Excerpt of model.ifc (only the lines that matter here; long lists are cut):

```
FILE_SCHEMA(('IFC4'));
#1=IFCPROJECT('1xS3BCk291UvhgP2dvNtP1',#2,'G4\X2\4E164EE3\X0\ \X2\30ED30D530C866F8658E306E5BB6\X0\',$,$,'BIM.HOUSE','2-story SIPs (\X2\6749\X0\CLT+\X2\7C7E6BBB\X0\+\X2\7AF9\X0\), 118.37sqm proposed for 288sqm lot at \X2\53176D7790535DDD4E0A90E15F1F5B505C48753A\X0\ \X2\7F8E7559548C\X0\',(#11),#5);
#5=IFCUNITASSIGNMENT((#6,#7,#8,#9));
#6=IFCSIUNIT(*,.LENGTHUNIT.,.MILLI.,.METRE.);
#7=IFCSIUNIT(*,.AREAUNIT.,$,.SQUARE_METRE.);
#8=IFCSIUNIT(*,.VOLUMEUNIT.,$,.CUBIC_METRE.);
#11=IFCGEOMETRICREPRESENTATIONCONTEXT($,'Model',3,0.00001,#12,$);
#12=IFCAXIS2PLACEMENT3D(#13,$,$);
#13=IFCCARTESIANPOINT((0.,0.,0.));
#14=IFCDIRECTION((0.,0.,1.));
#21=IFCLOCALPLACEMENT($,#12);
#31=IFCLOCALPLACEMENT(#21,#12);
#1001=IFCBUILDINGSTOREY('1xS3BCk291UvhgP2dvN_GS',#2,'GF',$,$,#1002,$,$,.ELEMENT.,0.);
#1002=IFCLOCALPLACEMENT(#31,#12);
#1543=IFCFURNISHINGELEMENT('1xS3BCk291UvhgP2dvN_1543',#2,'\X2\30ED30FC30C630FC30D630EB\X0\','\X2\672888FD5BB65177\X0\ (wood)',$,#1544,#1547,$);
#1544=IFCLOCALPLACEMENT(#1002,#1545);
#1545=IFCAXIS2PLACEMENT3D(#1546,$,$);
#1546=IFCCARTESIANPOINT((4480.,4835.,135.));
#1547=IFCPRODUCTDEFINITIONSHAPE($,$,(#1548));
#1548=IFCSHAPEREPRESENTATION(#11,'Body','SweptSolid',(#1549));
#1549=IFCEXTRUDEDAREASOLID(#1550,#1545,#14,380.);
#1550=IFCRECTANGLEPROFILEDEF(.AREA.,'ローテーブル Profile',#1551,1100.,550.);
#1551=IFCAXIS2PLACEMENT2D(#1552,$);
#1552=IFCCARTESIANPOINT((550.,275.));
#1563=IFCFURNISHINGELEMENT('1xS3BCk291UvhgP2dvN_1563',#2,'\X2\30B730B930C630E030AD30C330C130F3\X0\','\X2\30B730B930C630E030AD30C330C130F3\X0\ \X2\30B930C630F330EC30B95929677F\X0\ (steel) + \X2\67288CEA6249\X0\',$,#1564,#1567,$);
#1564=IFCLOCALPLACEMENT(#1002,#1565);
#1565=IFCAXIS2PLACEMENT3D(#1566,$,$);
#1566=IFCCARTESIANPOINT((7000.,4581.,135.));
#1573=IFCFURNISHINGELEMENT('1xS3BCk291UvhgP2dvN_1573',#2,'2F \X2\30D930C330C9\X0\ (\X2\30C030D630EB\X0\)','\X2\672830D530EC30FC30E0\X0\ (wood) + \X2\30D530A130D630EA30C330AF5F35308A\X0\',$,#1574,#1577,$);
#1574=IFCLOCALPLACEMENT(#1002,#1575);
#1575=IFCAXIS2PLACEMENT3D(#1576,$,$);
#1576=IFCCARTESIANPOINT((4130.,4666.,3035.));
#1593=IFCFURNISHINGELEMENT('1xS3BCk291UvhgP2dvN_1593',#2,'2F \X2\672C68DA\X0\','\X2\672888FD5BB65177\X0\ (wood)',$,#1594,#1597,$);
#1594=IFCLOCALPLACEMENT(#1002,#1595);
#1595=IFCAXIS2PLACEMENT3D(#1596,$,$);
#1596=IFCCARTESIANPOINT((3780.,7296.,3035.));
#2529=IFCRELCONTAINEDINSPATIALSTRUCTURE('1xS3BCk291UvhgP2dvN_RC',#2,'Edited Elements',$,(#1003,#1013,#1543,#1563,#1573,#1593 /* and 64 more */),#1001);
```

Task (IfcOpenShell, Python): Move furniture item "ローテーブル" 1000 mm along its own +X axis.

```python
import ifcopenshell
import ifcopenshell.api.geometry
import ifcopenshell.util.placement
import ifcopenshell.util.unit

model = ifcopenshell.open("model.ifc")
unit_scale = ifcopenshell.util.unit.calculate_unit_scale(model)

item = model.by_guid("1xS3BCk291UvhgP2dvN_1543")
matrix = ifcopenshell.util.placement.get_local_placement(item.ObjectPlacement)
matrix[:3, 3] += matrix[:3, 0] * 1 / unit_scale
ifcopenshell.api.geometry.edit_object_placement(model, product=item, matrix=matrix, is_si=False)

print(ifcopenshell.util.placement.get_local_placement(item.ObjectPlacement).round(3) + 0.0)

model.write("model-out.ifc")
```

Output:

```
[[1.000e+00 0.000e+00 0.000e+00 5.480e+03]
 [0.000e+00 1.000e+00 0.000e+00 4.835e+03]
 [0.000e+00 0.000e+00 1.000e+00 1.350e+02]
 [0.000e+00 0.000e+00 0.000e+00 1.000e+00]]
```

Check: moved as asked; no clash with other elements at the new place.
